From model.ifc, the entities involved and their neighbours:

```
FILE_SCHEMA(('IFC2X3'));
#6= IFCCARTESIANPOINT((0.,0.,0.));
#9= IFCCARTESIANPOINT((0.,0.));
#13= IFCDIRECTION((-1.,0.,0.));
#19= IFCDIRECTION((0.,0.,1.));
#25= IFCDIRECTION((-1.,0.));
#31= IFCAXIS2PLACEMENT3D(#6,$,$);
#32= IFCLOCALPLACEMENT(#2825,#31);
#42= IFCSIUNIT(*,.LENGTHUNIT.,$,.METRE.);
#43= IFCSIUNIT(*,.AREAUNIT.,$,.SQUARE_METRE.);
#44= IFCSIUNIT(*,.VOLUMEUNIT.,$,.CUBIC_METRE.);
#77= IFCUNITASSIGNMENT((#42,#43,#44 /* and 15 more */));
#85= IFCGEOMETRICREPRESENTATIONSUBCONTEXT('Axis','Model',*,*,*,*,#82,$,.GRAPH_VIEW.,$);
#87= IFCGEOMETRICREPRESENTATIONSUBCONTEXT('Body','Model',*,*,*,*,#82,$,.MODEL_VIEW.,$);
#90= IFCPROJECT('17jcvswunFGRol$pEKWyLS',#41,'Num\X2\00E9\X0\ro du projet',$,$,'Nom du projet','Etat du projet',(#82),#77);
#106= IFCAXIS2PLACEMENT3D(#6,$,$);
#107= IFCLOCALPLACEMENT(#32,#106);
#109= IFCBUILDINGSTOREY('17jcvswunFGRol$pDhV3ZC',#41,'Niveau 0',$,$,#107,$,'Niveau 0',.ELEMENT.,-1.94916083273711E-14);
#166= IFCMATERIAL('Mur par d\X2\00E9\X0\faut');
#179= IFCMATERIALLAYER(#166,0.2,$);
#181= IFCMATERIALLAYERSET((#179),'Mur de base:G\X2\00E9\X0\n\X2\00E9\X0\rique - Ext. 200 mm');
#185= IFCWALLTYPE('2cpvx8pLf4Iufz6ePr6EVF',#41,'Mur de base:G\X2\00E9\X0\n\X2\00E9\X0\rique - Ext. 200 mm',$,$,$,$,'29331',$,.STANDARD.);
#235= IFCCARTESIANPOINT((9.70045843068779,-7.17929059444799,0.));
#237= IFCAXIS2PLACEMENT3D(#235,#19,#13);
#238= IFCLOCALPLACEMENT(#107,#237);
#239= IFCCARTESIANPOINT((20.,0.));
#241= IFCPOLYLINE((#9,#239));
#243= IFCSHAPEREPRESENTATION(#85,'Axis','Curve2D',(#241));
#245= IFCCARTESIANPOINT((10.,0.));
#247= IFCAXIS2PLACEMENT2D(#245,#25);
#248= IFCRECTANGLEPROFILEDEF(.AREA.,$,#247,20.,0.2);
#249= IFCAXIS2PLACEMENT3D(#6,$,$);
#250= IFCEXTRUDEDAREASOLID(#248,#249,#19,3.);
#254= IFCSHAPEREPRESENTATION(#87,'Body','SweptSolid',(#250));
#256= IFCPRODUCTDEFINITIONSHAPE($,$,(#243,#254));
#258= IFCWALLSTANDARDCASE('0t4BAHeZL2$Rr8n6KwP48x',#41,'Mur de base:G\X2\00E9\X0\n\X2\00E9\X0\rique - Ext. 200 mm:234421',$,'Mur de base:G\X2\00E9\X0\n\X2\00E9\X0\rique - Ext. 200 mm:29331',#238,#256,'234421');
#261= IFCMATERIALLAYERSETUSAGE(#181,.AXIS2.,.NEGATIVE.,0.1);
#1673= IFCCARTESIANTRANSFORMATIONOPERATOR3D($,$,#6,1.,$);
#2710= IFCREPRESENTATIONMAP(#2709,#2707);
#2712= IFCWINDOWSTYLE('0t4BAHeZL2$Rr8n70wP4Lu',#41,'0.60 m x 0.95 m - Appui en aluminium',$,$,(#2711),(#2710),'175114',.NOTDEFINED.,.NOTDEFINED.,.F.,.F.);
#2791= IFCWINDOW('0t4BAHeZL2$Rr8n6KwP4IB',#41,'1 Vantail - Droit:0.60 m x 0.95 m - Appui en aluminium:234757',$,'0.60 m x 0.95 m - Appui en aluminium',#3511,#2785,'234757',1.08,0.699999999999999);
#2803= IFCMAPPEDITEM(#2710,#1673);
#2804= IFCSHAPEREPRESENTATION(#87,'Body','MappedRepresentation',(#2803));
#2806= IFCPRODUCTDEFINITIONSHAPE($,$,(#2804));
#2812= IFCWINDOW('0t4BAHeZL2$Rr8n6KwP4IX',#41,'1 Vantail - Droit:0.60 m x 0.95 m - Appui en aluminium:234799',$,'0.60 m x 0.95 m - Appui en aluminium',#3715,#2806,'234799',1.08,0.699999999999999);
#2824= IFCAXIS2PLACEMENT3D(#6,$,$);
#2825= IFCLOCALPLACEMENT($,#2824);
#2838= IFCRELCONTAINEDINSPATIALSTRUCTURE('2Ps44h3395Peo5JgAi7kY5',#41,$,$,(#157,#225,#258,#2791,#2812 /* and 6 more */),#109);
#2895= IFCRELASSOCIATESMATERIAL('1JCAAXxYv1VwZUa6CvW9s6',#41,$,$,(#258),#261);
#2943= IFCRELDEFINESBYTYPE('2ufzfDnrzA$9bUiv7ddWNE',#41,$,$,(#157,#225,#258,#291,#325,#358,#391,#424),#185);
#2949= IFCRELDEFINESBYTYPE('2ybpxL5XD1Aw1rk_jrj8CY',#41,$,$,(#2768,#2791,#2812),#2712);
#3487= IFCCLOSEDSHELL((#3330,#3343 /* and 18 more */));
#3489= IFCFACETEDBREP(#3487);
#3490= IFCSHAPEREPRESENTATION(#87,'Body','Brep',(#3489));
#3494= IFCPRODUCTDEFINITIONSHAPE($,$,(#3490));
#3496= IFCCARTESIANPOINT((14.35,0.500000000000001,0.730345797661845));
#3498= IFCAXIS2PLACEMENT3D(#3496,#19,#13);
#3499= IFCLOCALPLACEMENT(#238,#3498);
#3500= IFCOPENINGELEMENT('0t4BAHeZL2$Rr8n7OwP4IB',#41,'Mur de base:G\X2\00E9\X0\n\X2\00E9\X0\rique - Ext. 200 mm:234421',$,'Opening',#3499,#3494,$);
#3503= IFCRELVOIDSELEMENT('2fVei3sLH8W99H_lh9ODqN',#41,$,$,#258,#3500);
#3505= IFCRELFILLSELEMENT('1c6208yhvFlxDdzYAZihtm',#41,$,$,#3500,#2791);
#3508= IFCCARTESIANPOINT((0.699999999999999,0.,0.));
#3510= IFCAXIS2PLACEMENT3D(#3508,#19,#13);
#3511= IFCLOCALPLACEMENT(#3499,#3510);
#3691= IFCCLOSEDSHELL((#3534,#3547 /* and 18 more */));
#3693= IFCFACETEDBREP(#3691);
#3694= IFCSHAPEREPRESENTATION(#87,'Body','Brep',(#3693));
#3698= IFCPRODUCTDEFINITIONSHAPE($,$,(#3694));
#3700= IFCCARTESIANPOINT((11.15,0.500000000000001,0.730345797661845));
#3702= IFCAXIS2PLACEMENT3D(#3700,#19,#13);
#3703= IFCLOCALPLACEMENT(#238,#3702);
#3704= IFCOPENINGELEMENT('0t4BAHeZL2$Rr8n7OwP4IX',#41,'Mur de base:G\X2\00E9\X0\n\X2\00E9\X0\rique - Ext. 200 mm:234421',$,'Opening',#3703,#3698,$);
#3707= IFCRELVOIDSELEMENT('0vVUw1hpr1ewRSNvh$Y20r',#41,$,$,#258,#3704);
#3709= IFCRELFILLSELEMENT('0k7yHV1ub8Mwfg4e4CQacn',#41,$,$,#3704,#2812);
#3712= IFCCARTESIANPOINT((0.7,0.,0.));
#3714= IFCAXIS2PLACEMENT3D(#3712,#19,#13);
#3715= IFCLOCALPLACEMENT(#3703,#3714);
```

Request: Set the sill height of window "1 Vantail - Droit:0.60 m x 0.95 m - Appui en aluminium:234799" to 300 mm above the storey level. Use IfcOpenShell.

```python
import numpy as np
import ifcopenshell
import ifcopenshell.api.geometry
import ifcopenshell.geom
import ifcopenshell.util.element
import ifcopenshell.util.placement
import ifcopenshell.util.shape
import ifcopenshell.util.unit

model = ifcopenshell.open("model.ifc")
unit_scale = ifcopenshell.util.unit.calculate_unit_scale(model)

window = model.by_id(2812)
opening = window.FillsVoids[0].RelatingOpeningElement
storey = ifcopenshell.util.element.get_container(window, ifc_class="IfcBuildingStorey")
level = ifcopenshell.util.placement.get_local_placement(storey.ObjectPlacement)[2, 3]

# The opening's origin need not be at the sill, so measure its lowest point.
shape = ifcopenshell.geom.create_shape(ifcopenshell.geom.settings(), opening)
bottom = ifcopenshell.util.shape.get_shape_bottom_elevation(shape, shape.geometry) / unit_scale
dz = level + 0.3 - bottom

shift = np.array([0.0, 0.0, dz])
# The window is placed relative to its opening, so it follows when the opening moves.
matrix = ifcopenshell.util.placement.get_local_placement(opening.ObjectPlacement)
matrix[:3, 3] += shift
ifcopenshell.api.geometry.edit_object_placement(
    model, product=opening, matrix=matrix, is_si=False, should_transform_children=True
)

print(f"moved by {dz * unit_scale:+.3f} m")

model.write("model-out.ifc")
```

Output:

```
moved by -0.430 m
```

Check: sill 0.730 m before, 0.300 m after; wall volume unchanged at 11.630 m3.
